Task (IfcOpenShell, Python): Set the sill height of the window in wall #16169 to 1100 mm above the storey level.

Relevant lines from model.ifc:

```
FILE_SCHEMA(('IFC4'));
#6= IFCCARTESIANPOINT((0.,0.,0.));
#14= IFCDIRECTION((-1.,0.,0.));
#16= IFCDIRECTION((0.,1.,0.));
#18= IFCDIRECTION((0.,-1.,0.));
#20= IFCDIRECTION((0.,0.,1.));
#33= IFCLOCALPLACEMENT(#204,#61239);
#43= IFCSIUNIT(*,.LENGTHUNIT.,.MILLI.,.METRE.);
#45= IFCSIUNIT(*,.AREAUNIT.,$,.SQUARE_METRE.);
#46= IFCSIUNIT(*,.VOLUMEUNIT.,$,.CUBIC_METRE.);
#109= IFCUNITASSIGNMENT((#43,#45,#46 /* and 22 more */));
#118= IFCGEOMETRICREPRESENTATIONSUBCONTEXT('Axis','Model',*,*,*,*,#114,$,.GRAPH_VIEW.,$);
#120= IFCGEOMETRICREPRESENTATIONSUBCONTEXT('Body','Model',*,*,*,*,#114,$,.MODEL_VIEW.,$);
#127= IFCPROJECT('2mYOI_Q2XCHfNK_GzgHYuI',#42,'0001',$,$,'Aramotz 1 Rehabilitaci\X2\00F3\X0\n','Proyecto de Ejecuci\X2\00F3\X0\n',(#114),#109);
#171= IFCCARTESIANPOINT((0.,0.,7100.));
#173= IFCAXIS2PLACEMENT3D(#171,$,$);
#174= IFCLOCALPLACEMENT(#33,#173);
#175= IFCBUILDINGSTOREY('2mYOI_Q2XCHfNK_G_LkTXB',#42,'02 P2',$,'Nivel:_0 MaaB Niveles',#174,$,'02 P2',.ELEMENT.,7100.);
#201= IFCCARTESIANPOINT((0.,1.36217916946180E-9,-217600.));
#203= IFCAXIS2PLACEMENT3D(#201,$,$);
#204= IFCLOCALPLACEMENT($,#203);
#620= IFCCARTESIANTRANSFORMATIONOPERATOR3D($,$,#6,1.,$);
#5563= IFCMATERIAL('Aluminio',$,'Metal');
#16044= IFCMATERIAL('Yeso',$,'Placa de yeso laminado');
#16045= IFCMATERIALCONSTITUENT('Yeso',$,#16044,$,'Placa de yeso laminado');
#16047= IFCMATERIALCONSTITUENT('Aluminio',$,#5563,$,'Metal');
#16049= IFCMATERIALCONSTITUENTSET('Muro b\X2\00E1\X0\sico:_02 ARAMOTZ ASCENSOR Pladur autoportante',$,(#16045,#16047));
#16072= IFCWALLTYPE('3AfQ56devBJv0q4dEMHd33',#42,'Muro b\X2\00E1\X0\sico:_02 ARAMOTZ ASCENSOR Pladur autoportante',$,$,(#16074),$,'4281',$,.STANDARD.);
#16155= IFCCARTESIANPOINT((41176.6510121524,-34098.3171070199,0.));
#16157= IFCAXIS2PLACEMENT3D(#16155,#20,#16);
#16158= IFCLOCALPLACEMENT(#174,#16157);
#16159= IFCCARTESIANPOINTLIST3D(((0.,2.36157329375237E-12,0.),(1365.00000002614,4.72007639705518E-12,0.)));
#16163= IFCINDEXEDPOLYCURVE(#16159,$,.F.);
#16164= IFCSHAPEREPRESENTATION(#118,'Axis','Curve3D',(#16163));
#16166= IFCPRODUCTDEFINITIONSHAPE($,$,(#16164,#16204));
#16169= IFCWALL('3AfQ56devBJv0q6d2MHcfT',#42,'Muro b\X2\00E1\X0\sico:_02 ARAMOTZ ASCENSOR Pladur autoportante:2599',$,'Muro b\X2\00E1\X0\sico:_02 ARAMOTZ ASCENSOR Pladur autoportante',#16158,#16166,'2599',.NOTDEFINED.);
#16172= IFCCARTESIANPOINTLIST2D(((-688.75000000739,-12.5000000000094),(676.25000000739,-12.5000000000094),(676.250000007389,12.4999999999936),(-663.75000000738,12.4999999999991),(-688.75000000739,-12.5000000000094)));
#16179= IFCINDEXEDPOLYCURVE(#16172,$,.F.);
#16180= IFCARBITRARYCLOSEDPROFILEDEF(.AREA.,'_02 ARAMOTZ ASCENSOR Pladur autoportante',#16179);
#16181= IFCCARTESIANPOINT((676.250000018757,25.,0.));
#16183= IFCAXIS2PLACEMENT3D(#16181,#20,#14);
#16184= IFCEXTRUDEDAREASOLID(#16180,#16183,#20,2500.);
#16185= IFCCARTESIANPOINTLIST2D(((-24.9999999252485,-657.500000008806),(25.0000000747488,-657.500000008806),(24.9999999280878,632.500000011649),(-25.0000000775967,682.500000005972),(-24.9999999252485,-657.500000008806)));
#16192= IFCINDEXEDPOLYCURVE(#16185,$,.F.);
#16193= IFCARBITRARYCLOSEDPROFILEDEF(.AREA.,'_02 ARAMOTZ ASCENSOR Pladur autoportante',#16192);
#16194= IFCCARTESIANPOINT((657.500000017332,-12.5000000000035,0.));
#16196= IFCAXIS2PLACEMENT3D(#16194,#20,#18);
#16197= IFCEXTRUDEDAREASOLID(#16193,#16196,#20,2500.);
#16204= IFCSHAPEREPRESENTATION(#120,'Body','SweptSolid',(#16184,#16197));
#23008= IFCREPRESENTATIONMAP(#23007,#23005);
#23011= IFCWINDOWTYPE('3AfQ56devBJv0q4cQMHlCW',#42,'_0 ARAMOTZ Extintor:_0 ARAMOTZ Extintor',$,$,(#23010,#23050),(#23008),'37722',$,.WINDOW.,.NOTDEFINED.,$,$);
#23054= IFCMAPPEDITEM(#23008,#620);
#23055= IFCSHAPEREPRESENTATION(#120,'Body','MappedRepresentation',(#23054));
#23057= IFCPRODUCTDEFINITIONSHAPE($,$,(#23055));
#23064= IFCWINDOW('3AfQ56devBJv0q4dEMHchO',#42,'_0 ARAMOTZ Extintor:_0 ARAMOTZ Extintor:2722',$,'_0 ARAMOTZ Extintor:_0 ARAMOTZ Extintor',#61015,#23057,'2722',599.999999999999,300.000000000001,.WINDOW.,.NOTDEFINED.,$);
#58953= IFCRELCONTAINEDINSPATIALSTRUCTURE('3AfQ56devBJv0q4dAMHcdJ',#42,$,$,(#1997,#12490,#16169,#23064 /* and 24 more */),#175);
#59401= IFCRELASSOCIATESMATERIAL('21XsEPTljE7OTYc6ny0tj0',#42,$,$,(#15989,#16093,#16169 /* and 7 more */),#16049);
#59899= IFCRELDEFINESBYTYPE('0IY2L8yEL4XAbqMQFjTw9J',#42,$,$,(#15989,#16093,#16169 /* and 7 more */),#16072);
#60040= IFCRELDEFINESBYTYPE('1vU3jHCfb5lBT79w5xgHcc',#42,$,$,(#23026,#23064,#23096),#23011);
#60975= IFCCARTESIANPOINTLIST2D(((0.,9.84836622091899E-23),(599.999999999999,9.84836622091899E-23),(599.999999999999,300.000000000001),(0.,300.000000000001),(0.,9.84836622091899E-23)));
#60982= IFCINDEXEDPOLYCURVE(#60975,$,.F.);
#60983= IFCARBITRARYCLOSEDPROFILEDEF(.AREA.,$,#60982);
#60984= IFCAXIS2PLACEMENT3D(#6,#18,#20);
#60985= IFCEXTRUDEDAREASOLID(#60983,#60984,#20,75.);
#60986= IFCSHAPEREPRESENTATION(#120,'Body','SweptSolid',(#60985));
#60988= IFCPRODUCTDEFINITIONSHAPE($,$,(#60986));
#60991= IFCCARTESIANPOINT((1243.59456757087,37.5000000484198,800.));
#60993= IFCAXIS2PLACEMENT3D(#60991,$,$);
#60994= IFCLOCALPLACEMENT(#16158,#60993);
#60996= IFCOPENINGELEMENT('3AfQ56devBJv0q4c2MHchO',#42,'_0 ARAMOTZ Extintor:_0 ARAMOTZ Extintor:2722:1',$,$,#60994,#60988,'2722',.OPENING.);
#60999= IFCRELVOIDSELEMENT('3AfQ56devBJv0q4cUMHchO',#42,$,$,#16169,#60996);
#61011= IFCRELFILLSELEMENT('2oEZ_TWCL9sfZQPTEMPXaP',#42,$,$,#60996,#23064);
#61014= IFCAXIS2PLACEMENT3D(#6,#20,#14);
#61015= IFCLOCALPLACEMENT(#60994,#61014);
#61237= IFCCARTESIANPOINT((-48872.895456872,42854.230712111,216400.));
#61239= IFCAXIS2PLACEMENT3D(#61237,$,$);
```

```python
import numpy as np
import ifcopenshell
import ifcopenshell.api.geometry
import ifcopenshell.geom
import ifcopenshell.util.element
import ifcopenshell.util.placement
import ifcopenshell.util.shape
import ifcopenshell.util.unit

model = ifcopenshell.open("model.ifc")
unit_scale = ifcopenshell.util.unit.calculate_unit_scale(model)

window = model.by_guid("3AfQ56devBJv0q4dEMHchO")
opening = window.FillsVoids[0].RelatingOpeningElement
storey = ifcopenshell.util.element.get_container(window, ifc_class="IfcBuildingStorey")
level = ifcopenshell.util.placement.get_local_placement(storey.ObjectPlacement)[2, 3]

# The opening's origin need not be at the sill, so measure its lowest point.
shape = ifcopenshell.geom.create_shape(ifcopenshell.geom.settings(), opening)
bottom = ifcopenshell.util.shape.get_shape_bottom_elevation(shape, shape.geometry) / unit_scale
dz = level + 1100.0 - bottom

shift = np.array([0.0, 0.0, dz])
# The window is placed relative to its opening, so it follows when the opening moves.
matrix = ifcopenshell.util.placement.get_local_placement(opening.ObjectPlacement)
matrix[:3, 3] += shift
ifcopenshell.api.geometry.edit_object_placement(
    model, product=opening, matrix=matrix, is_si=False, should_transform_children=True
)

print(f"moved by {dz * unit_scale:+.3f} m")

model.write("model_v2.ifc")
```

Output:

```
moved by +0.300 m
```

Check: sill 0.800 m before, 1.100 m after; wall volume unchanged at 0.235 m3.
